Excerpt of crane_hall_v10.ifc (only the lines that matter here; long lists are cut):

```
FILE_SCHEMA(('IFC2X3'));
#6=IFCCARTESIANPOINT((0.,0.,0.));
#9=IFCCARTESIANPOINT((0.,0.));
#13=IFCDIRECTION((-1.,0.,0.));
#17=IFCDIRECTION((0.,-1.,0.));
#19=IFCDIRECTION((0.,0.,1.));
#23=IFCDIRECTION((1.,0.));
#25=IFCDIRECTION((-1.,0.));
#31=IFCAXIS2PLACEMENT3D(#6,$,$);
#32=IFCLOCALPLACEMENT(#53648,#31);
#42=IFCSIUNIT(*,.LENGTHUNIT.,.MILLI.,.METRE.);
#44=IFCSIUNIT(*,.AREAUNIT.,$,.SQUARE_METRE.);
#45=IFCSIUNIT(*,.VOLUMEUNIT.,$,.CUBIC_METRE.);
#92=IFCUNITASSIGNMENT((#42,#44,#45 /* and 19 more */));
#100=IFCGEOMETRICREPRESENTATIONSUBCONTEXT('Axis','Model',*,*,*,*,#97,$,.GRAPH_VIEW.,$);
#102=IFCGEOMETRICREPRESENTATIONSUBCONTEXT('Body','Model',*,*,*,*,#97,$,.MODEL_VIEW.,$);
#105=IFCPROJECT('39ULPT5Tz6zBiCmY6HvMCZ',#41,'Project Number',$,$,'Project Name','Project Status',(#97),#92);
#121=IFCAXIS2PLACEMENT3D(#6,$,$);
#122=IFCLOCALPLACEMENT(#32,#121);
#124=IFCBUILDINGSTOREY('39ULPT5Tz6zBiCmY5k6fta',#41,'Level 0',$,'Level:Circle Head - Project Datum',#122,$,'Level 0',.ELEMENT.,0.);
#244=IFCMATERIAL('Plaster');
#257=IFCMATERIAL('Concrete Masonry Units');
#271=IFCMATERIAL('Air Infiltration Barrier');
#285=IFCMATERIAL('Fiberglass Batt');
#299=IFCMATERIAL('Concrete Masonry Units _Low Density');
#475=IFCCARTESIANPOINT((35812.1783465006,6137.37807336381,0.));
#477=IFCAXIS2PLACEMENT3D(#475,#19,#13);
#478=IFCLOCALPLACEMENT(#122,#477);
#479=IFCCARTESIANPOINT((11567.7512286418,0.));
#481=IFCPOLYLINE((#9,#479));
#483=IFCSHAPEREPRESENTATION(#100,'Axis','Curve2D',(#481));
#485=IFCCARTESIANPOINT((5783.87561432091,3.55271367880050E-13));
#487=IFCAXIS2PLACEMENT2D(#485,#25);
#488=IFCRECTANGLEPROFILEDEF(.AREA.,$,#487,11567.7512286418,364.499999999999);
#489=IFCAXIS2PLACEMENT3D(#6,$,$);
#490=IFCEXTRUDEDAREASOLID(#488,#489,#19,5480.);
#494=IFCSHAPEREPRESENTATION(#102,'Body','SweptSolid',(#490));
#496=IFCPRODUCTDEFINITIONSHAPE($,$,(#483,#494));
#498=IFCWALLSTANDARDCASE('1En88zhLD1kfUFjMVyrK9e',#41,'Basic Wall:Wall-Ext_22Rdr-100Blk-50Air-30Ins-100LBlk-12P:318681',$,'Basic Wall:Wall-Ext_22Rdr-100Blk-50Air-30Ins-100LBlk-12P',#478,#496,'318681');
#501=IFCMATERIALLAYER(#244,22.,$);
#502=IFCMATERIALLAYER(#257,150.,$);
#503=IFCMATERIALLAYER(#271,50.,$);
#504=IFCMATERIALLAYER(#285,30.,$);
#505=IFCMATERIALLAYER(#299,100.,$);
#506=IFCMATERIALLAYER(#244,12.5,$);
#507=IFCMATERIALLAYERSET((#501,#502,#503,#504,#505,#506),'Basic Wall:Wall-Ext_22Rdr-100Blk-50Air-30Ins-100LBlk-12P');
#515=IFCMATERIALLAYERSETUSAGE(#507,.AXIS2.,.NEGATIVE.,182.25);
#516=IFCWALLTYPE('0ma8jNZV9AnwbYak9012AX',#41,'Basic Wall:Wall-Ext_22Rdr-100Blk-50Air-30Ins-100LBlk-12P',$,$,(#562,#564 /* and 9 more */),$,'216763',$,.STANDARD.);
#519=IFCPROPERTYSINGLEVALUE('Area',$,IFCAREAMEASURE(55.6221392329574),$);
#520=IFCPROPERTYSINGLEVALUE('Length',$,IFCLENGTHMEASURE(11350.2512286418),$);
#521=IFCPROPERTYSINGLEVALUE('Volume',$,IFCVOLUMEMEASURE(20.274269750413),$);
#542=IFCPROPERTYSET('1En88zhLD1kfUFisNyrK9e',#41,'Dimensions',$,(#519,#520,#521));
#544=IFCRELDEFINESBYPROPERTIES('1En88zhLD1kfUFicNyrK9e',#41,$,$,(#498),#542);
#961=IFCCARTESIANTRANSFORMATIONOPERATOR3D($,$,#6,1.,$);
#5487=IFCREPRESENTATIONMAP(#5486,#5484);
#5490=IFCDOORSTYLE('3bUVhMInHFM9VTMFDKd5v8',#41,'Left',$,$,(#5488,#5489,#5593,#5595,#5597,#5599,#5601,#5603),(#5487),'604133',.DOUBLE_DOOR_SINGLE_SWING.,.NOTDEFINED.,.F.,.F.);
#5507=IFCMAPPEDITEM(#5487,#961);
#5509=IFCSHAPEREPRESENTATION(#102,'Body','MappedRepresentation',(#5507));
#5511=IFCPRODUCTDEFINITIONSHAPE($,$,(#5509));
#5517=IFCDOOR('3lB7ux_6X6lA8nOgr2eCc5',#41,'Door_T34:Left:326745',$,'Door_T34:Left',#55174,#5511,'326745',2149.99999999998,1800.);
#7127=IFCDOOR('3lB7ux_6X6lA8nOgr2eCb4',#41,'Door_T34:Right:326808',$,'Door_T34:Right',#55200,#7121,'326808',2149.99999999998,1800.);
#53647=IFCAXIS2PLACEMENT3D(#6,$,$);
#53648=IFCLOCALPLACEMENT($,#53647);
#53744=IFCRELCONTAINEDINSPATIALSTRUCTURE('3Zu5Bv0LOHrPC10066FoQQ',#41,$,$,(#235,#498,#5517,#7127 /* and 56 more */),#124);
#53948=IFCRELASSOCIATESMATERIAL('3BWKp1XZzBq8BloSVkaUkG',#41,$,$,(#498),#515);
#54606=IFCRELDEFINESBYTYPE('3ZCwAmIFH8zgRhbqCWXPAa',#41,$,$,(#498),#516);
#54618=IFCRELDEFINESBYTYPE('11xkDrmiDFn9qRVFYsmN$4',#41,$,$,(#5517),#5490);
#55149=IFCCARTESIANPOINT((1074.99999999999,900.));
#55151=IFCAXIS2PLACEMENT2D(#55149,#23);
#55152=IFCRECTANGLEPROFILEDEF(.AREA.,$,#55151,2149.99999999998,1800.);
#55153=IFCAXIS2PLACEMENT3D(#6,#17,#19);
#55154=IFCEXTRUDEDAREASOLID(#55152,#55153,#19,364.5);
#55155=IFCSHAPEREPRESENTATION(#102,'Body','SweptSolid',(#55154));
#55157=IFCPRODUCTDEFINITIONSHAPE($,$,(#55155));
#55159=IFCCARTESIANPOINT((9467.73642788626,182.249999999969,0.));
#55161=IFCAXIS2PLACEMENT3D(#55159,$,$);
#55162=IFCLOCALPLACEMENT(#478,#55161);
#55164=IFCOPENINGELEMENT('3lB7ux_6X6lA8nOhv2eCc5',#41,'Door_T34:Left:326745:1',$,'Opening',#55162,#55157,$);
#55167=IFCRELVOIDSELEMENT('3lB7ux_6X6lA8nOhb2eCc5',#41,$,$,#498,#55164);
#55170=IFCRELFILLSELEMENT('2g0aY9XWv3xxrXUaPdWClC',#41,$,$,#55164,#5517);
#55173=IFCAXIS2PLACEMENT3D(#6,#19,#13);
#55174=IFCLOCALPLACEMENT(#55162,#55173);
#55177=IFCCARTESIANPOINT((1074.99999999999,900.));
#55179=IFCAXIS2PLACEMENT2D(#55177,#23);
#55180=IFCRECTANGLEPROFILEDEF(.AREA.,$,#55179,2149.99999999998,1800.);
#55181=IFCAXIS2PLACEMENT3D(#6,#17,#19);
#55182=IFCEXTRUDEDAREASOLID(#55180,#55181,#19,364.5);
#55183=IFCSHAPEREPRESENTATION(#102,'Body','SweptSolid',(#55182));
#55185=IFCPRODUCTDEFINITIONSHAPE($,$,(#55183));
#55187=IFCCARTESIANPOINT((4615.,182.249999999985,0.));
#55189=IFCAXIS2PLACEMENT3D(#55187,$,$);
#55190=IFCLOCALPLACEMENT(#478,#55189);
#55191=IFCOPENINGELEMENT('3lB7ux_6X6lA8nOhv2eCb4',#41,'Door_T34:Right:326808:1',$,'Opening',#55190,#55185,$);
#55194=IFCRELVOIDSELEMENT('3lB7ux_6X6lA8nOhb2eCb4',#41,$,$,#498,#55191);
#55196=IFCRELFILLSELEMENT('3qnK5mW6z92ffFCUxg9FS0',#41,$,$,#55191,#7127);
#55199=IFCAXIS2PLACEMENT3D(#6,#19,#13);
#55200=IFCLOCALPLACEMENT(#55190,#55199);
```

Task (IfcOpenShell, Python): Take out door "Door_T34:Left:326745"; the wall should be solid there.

```python
import ifcopenshell
import ifcopenshell.api.feature
import ifcopenshell.api.pset
import ifcopenshell.api.root
import ifcopenshell.geom
import ifcopenshell.util.element
import ifcopenshell.util.shape
import ifcopenshell.util.unit

model = ifcopenshell.open("crane_hall_v10.ifc")
area_scale = ifcopenshell.util.unit.calculate_unit_scale(model, "AREAUNIT")
volume_scale = ifcopenshell.util.unit.calculate_unit_scale(model, "VOLUMEUNIT")
settings = ifcopenshell.geom.settings()


def volume(element):
    """Net volume in cubic metres, openings subtracted."""
    shape = ifcopenshell.geom.create_shape(settings, element)
    return ifcopenshell.util.shape.get_volume(shape.geometry)


door = model.by_guid("3lB7ux_6X6lA8nOgr2eCc5")
opening = door.FillsVoids[0].RelatingOpeningElement
wall = opening.VoidsElements[0].RelatingBuildingElement
before = volume(wall)

ifcopenshell.api.root.remove_product(model, product=door)
ifcopenshell.api.feature.remove_feature(model, feature=opening)

after = volume(wall)
thickness = 0.3645  # wall thickness in metres

# Update the wall's stored quantities.
pset = model.by_id(ifcopenshell.util.element.get_pset(wall, "Dimensions", should_inherit=False)["id"])
ifcopenshell.api.pset.edit_pset(model, pset=pset, properties={
    "Area": model.create_entity("IfcAreaMeasure", after / thickness / area_scale),
    "Volume": model.create_entity("IfcVolumeMeasure", after / volume_scale),
})

print(f"wall volume {before:.3f} -> {after:.3f} m3")

model.write("crane_hall_v10_v2.ifc")
```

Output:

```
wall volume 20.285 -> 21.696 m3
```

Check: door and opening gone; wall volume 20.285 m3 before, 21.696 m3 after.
